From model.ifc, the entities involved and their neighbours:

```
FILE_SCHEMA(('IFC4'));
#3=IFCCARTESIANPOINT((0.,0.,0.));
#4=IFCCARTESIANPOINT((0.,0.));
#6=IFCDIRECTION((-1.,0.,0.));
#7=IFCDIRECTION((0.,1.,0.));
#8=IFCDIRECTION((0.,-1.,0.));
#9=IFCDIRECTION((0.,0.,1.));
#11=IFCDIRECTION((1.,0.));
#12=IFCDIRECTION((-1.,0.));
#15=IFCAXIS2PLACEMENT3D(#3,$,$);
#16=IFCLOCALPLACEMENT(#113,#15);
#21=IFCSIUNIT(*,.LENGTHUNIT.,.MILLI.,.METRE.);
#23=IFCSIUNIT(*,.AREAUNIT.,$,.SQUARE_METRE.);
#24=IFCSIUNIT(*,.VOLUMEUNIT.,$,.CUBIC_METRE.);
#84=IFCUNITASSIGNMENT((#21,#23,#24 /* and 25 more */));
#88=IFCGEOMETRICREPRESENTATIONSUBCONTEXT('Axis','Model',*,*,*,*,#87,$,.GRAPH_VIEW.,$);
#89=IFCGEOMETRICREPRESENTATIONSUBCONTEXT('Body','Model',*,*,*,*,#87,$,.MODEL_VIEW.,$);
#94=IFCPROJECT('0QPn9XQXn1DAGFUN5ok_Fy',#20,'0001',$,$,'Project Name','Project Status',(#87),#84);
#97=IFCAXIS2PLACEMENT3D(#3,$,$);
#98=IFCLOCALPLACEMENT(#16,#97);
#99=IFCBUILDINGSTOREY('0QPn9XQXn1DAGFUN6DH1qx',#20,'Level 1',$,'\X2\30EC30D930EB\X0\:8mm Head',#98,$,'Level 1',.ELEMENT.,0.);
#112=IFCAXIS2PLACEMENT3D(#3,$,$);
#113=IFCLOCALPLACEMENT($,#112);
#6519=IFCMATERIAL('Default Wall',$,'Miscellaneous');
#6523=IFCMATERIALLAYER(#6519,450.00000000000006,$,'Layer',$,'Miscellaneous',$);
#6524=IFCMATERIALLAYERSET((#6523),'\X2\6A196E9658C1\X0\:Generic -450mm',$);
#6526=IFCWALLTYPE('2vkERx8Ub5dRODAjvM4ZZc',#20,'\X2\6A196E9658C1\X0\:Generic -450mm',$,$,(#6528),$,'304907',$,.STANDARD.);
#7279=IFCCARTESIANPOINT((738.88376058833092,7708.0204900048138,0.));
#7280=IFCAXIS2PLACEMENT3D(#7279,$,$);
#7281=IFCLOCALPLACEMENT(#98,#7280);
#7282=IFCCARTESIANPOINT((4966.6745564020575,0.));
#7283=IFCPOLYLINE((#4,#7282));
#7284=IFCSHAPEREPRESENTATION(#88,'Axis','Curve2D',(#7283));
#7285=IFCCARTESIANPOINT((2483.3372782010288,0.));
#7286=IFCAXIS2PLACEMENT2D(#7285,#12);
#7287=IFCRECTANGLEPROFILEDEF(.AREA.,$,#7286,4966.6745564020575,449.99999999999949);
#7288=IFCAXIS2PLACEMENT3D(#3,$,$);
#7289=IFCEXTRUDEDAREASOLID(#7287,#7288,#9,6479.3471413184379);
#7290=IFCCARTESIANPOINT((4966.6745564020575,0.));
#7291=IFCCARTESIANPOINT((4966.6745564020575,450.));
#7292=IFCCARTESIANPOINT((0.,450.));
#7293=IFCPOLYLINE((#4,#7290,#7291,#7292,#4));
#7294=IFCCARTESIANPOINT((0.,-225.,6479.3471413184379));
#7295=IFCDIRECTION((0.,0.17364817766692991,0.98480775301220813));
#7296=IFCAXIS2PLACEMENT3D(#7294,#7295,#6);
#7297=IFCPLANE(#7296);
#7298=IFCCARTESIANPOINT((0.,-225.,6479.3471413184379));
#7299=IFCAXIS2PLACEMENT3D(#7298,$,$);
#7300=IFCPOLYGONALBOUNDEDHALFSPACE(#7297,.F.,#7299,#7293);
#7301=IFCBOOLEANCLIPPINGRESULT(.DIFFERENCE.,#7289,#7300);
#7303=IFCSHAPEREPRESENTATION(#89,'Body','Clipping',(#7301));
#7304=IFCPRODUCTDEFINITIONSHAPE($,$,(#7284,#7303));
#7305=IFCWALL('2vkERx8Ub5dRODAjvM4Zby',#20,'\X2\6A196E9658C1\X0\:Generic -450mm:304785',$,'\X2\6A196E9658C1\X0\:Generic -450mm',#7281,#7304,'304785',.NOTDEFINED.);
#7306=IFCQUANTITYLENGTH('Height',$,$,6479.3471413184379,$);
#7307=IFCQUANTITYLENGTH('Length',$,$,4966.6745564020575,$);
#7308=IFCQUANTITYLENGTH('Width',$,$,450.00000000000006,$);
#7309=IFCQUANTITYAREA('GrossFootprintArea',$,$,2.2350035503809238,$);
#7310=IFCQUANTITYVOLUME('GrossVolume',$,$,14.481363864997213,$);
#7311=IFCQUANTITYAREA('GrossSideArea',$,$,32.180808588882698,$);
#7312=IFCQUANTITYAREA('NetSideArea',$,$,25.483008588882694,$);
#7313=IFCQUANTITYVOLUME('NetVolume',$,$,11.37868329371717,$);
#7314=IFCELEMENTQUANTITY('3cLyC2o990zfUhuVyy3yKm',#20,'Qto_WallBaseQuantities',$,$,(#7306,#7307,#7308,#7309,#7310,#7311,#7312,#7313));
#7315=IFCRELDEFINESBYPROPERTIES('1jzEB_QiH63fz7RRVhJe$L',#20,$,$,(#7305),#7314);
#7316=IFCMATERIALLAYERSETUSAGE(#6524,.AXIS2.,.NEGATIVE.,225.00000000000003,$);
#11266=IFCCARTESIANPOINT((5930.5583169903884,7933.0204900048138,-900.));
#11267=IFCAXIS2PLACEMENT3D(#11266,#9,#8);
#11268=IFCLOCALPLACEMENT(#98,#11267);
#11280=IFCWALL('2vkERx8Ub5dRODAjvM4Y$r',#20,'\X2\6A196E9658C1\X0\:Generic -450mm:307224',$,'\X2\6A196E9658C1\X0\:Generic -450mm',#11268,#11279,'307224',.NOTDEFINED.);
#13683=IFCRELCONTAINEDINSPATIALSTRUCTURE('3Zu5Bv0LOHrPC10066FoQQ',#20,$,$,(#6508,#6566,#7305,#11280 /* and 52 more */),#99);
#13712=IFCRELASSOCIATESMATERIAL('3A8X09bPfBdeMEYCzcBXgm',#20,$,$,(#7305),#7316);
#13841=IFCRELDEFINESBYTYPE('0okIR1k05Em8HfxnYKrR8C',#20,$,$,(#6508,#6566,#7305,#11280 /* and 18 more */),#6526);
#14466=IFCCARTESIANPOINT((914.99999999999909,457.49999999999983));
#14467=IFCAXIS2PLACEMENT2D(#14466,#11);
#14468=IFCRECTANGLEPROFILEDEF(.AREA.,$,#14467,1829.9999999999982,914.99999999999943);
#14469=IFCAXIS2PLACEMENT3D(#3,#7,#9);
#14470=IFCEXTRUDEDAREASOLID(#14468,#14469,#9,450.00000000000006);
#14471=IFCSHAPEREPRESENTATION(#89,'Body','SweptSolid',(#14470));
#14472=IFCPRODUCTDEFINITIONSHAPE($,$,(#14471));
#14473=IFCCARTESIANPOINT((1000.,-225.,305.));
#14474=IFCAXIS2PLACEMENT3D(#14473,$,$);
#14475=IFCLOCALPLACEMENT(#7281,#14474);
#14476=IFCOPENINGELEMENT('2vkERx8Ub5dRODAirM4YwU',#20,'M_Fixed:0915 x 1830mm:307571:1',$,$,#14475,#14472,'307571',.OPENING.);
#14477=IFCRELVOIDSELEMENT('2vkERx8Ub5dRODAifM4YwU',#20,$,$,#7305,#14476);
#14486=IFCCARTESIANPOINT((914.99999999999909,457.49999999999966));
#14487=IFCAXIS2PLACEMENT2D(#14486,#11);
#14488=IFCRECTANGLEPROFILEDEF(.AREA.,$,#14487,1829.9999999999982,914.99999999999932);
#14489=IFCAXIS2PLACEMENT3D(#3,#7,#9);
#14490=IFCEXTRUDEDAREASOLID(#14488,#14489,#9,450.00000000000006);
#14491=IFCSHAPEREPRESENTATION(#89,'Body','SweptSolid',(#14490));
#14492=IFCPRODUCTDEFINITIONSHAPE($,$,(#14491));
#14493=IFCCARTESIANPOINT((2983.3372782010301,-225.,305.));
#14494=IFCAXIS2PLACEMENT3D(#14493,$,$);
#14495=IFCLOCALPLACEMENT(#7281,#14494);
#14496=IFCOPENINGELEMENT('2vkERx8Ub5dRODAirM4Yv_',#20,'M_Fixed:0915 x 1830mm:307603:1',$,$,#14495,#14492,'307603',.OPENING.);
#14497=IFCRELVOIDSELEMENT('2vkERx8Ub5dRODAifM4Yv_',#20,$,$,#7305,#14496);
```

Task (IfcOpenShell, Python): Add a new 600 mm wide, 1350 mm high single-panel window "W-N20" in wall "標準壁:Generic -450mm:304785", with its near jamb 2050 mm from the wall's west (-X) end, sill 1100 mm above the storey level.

```python
import numpy as np
import ifcopenshell
import ifcopenshell.api.feature
import ifcopenshell.api.geometry
import ifcopenshell.api.pset
import ifcopenshell.api.root
import ifcopenshell.api.spatial
import ifcopenshell.geom
import ifcopenshell.util.element
import ifcopenshell.util.placement
import ifcopenshell.util.representation
import ifcopenshell.util.shape
import ifcopenshell.util.unit

model = ifcopenshell.open("model.ifc")
unit_scale = ifcopenshell.util.unit.calculate_unit_scale(model)
area_scale = ifcopenshell.util.unit.calculate_unit_scale(model, "AREAUNIT")
volume_scale = ifcopenshell.util.unit.calculate_unit_scale(model, "VOLUMEUNIT")
settings = ifcopenshell.geom.settings()


def volume(element):
    """Net volume in cubic metres, openings subtracted."""
    shape = ifcopenshell.geom.create_shape(settings, element)
    return ifcopenshell.util.shape.get_volume(shape.geometry)


wall = model.by_guid("2vkERx8Ub5dRODAjvM4Zby")
storey = ifcopenshell.util.element.get_container(wall, ifc_class="IfcBuildingStorey")
context = ifcopenshell.util.representation.get_context(model, "Model", "Body", "MODEL_VIEW")
before = volume(wall)

width, height, from_end, sill = 0.6, 1.35, 2.05, 1.1  # metres

# The wall runs along its own X axis, and the end named is its -X end.
wall_shape = ifcopenshell.geom.create_shape(settings, wall)
x, y, z = ifcopenshell.util.shape.get_vertices(wall_shape.geometry).T
start = x.min() + from_end
face, thickness = float(y.min()), float(y.max() - y.min())
wall_matrix = ifcopenshell.util.placement.get_local_placement(wall.ObjectPlacement)
level = ifcopenshell.util.placement.get_local_placement(storey.ObjectPlacement)[2, 3]


def in_wall(x, y):
    """Placement at x, y metres in the wall's axes, at sill height."""
    matrix = wall_matrix.copy()
    matrix[:, 3] = wall_matrix @ np.array([x / unit_scale, y / unit_scale, 0.0, 1.0])
    matrix[2, 3] = level + sill / unit_scale
    return matrix


# Opening: a box that overshoots both wall faces by 50 mm.
opening = ifcopenshell.api.root.create_entity(model, ifc_class="IfcOpeningElement", predefined_type="OPENING")
box = ifcopenshell.api.geometry.add_wall_representation(
    model, context=context, length=width, height=height, thickness=thickness + 0.1
)
ifcopenshell.api.geometry.assign_representation(model, product=opening, representation=box)
ifcopenshell.api.geometry.edit_object_placement(model, product=opening, matrix=in_wall(start, face - 0.05), is_si=False)
ifcopenshell.api.feature.add_feature(model, feature=opening, element=wall)

window = ifcopenshell.api.root.create_entity(model, ifc_class="IfcWindow", name="W-N20", predefined_type="WINDOW")
window.OverallWidth, window.OverallHeight = width / unit_scale, height / unit_scale
window.PartitioningType = "SINGLE_PANEL"
body = ifcopenshell.api.geometry.add_window_representation(
    model,
    context=context,
    overall_width=window.OverallWidth,
    overall_height=window.OverallHeight,
    partition_type="SINGLE_PANEL",
)
ifcopenshell.api.geometry.assign_representation(model, product=window, representation=body)
ifcopenshell.api.spatial.assign_container(model, products=[window], relating_structure=storey)
ifcopenshell.api.feature.add_filling(model, opening=opening, element=window)

# Centre the window in the wall's thickness.
ifcopenshell.api.geometry.edit_object_placement(model, product=window, matrix=in_wall(start, face), is_si=False)
window_shape = ifcopenshell.geom.create_shape(settings, window)
depth = ifcopenshell.util.shape.get_vertices(window_shape.geometry)[:, 1]
offset = face + thickness / 2 - (depth.min() + depth.max()) / 2
ifcopenshell.api.geometry.edit_object_placement(model, product=window, matrix=in_wall(start, offset), is_si=False)

after = volume(wall)

# Update the wall's stored quantities.
qto = model.by_id(ifcopenshell.util.element.get_pset(wall, "Qto_WallBaseQuantities", should_inherit=False)["id"])
ifcopenshell.api.pset.edit_qto(model, qto=qto, properties={
    "NetSideArea": after / thickness / area_scale,
    "NetVolume": after / volume_scale,
})

print(f"wall volume {before:.3f} -> {after:.3f} m3")

model.write("model-out.ifc")
```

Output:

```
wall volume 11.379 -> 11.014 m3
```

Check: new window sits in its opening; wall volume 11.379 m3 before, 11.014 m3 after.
